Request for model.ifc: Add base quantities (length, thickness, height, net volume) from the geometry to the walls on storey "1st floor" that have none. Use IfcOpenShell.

First a look at what the model holds.

```python
import ifcopenshell
import ifcopenshell.util.element
import ifcopenshell.util.unit

model = ifcopenshell.open("model.ifc")
print(model.schema)
for unit_type in ("LENGTHUNIT", "AREAUNIT", "VOLUMEUNIT"):
    print(unit_type, ifcopenshell.util.unit.calculate_unit_scale(model, unit_type))
storey = next(s for s in model.by_type("IfcBuildingStorey") if s.Name == "1st floor")
walls = [e for e in ifcopenshell.util.element.get_decomposition(storey) if e.is_a("IfcWall")]
for e in sorted(walls, key=lambda e: e.id()):
    print(e.id(), e.is_a(), e.Name, list(ifcopenshell.util.element.get_psets(e, qtos_only=True)), sep=" | ")
```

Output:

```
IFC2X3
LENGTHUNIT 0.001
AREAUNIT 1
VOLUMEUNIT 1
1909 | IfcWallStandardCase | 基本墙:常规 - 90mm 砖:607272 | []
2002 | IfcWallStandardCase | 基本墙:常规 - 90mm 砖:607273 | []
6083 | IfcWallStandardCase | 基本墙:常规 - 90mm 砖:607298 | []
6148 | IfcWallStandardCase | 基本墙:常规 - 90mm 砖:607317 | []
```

```python
import ifcopenshell
import ifcopenshell.api.pset
import ifcopenshell.geom
import ifcopenshell.util.element
import ifcopenshell.util.shape
import ifcopenshell.util.unit

model = ifcopenshell.open("model.ifc")
unit_scale = ifcopenshell.util.unit.calculate_unit_scale(model)
volume_scale = ifcopenshell.util.unit.calculate_unit_scale(model, "VOLUMEUNIT")
settings = ifcopenshell.geom.settings()

storey = next(s for s in model.by_type("IfcBuildingStorey") if s.Name == "1st floor")
walls = [e for e in ifcopenshell.util.element.get_decomposition(storey) if e.is_a("IfcWall")]

for e in sorted(walls, key=lambda e: e.id()):
    if ifcopenshell.util.element.get_psets(e, qtos_only=True, should_inherit=False):
        continue
    # Geometry comes back in metres, in the element's own axes.
    shape = ifcopenshell.geom.create_shape(settings, e)
    values = {
        "Length": ifcopenshell.util.shape.get_x(shape.geometry) / unit_scale,
        "Width": ifcopenshell.util.shape.get_y(shape.geometry) / unit_scale,
        "Height": ifcopenshell.util.shape.get_z(shape.geometry) / unit_scale,
        "NetVolume": ifcopenshell.util.shape.get_volume(shape.geometry) / volume_scale,
    }
    qto = ifcopenshell.api.pset.add_qto(model, product=e, name="BaseQuantities")
    ifcopenshell.api.pset.edit_qto(model, qto=qto, properties=values)
    print(e.id(), {k: round(v, 3) for k, v in values.items()})

model.write("model-out.ifc")
```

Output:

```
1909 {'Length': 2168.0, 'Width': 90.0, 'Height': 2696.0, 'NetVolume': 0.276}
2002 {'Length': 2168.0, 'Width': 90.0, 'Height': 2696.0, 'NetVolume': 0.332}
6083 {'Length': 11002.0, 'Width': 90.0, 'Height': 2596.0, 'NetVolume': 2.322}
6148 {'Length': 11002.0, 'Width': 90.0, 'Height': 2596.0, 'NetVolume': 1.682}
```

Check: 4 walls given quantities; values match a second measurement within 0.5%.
